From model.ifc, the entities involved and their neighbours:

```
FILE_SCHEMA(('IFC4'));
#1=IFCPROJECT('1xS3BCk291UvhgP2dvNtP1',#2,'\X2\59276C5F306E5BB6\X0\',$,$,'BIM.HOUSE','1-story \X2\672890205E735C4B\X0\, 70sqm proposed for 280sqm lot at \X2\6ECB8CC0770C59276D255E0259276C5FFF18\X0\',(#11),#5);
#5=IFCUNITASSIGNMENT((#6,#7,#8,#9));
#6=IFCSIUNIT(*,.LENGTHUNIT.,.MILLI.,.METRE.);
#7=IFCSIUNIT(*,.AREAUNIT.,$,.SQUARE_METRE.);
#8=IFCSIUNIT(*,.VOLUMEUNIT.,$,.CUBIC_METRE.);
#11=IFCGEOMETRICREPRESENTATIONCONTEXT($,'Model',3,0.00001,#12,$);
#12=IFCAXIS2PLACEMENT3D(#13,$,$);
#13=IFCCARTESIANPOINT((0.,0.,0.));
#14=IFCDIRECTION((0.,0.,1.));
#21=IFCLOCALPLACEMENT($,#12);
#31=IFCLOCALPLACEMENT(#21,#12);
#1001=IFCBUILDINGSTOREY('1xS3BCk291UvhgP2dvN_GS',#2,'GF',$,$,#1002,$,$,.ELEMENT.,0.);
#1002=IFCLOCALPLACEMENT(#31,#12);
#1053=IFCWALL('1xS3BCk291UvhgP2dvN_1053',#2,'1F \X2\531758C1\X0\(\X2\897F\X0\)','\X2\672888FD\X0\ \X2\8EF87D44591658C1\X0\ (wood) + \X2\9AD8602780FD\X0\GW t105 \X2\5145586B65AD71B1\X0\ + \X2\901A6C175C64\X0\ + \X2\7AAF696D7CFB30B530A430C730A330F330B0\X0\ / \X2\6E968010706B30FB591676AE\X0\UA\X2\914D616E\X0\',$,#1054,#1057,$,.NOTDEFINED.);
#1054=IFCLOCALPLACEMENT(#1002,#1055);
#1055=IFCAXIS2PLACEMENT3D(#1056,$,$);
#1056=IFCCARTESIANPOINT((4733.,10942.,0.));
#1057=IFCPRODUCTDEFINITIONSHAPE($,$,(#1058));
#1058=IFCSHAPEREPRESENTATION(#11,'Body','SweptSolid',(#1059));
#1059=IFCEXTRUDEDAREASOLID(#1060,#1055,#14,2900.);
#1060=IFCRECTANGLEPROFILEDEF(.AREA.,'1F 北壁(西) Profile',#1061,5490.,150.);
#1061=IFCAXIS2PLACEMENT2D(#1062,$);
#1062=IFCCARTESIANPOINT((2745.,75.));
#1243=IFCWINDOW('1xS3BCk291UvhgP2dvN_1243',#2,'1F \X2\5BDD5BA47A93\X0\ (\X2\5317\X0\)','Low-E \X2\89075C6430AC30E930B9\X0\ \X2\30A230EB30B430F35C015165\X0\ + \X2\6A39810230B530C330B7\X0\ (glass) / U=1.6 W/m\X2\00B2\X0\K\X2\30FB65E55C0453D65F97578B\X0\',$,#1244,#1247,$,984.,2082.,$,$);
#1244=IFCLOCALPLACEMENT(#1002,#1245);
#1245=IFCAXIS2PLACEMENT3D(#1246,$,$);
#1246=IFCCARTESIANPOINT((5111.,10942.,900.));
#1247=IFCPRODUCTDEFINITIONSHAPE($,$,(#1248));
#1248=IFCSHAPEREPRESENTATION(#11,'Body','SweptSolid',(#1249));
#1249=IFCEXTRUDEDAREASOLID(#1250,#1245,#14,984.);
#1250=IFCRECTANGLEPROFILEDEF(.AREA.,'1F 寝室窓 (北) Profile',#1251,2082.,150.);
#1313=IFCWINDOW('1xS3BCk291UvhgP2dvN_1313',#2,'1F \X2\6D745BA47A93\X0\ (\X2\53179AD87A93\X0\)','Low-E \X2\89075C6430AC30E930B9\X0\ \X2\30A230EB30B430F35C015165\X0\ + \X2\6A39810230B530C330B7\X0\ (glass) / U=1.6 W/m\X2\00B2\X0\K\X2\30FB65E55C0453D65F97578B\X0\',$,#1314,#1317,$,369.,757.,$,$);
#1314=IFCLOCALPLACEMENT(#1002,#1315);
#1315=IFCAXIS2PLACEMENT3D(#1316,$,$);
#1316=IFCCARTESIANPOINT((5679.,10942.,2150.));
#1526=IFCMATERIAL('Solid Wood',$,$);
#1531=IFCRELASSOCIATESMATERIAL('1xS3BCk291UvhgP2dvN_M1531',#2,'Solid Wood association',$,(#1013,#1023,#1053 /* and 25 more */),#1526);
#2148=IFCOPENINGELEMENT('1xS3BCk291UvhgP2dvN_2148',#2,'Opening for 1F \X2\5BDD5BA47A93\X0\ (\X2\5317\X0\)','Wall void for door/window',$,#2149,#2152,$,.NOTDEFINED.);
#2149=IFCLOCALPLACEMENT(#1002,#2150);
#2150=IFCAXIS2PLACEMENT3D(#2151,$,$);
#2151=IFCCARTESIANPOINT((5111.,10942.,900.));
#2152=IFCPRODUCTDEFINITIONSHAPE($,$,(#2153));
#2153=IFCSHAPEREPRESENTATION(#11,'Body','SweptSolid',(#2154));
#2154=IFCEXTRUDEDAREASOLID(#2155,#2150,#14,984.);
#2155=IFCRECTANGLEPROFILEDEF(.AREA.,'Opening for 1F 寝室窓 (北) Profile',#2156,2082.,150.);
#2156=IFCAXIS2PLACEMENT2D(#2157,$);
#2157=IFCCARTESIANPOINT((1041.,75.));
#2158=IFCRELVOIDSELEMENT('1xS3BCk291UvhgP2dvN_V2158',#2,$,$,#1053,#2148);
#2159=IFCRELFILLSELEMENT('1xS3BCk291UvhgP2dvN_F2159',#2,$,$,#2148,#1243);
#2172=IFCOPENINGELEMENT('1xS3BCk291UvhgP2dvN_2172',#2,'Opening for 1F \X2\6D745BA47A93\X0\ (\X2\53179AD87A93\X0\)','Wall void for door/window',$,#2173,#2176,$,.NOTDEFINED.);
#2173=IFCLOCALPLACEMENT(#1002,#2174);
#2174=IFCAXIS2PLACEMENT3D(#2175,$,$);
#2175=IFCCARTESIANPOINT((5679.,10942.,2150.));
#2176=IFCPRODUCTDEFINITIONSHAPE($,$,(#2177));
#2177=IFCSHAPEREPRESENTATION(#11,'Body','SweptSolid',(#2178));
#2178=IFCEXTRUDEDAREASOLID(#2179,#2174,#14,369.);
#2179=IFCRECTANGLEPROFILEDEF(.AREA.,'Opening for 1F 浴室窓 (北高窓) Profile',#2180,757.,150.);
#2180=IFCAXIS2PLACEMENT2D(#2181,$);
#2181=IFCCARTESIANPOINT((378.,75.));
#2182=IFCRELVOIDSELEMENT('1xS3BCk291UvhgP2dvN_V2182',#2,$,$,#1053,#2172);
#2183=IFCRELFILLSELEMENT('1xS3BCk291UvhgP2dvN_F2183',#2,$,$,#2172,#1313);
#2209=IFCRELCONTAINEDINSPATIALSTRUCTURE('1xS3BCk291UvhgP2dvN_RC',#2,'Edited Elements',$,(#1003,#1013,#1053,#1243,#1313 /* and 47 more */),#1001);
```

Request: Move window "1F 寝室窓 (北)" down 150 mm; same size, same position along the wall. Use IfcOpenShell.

```python
import numpy as np
import ifcopenshell
import ifcopenshell.api.geometry
import ifcopenshell.util.placement
import ifcopenshell.util.unit

model = ifcopenshell.open("model.ifc")
unit_scale = ifcopenshell.util.unit.calculate_unit_scale(model)

window = model.by_guid("1xS3BCk291UvhgP2dvN_1243")
opening = window.FillsVoids[0].RelatingOpeningElement
dz = -0.15 / unit_scale

shift = np.array([0.0, 0.0, dz])
# The window is not placed relative to its opening, so move both.
for product in (opening, window):
    matrix = ifcopenshell.util.placement.get_local_placement(product.ObjectPlacement)
    matrix[:3, 3] += shift
    ifcopenshell.api.geometry.edit_object_placement(model, product=product, matrix=matrix, is_si=False)

print(f"moved by {dz * unit_scale:+.3f} m")

model.write("model_updated.ifc")
```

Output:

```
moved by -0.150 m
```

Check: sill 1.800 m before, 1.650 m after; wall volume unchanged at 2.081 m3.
